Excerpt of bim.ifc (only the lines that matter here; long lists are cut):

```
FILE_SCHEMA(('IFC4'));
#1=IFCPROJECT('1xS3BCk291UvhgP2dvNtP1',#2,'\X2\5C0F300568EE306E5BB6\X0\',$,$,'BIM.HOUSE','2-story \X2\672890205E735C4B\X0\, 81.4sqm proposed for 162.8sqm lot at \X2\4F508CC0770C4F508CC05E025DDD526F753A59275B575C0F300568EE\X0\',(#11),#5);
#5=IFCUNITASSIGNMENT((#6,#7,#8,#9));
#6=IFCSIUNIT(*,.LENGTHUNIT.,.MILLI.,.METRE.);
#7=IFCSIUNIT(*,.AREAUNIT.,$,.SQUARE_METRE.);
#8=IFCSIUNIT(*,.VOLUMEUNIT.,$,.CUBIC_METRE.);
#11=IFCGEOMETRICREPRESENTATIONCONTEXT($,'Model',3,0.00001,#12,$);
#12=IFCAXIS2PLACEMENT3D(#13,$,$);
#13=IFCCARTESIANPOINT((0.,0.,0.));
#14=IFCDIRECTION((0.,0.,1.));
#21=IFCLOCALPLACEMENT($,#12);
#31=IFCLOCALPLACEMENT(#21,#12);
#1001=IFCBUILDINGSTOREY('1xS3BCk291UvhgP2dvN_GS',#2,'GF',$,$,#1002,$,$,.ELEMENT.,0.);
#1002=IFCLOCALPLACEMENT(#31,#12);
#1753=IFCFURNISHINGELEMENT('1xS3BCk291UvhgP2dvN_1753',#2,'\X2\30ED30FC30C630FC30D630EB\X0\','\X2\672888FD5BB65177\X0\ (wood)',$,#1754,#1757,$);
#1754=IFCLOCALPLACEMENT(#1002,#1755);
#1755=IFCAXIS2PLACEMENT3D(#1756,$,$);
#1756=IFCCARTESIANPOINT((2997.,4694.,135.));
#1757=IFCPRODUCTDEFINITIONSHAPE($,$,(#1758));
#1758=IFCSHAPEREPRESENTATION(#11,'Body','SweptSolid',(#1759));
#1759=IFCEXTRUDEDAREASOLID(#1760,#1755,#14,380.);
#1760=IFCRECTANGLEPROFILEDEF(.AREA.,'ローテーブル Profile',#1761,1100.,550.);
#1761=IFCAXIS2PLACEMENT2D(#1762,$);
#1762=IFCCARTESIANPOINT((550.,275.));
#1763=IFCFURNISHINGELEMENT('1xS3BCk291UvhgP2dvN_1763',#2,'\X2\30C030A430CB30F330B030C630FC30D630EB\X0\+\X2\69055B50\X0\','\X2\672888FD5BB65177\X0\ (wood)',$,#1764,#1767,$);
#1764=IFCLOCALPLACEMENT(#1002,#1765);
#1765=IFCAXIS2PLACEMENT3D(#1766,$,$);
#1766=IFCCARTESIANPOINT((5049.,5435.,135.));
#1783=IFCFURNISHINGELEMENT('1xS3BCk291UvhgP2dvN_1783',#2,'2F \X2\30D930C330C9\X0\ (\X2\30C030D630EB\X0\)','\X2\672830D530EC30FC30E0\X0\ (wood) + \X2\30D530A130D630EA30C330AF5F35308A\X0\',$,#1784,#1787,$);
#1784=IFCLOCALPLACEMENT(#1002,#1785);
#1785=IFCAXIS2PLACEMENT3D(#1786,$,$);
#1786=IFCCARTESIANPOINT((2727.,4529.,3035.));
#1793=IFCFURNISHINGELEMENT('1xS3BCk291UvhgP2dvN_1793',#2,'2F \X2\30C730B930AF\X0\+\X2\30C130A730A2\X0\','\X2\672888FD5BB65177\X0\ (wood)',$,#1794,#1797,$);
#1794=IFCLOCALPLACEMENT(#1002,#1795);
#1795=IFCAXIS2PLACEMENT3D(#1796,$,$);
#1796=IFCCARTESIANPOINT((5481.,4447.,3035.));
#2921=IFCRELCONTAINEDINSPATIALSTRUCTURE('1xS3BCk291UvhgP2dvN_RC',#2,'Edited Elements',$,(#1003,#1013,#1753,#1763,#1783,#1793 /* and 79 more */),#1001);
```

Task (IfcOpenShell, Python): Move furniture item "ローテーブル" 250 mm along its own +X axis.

```python
import ifcopenshell
import ifcopenshell.api.geometry
import ifcopenshell.util.placement

model = ifcopenshell.open("bim.ifc")

item = model.by_guid("1xS3BCk291UvhgP2dvN_1753")
matrix = ifcopenshell.util.placement.get_local_placement(item.ObjectPlacement)
matrix[:3, 3] += matrix[:3, 0] * 250.0
ifcopenshell.api.geometry.edit_object_placement(model, product=item, matrix=matrix, is_si=False)

print(ifcopenshell.util.placement.get_local_placement(item.ObjectPlacement).round(3) + 0.0)

model.write("bim_v2.ifc")
```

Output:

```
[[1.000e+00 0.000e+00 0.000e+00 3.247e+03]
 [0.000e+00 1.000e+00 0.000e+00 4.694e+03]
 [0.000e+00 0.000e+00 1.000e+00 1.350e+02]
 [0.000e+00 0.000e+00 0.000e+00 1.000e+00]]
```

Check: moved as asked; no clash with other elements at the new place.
